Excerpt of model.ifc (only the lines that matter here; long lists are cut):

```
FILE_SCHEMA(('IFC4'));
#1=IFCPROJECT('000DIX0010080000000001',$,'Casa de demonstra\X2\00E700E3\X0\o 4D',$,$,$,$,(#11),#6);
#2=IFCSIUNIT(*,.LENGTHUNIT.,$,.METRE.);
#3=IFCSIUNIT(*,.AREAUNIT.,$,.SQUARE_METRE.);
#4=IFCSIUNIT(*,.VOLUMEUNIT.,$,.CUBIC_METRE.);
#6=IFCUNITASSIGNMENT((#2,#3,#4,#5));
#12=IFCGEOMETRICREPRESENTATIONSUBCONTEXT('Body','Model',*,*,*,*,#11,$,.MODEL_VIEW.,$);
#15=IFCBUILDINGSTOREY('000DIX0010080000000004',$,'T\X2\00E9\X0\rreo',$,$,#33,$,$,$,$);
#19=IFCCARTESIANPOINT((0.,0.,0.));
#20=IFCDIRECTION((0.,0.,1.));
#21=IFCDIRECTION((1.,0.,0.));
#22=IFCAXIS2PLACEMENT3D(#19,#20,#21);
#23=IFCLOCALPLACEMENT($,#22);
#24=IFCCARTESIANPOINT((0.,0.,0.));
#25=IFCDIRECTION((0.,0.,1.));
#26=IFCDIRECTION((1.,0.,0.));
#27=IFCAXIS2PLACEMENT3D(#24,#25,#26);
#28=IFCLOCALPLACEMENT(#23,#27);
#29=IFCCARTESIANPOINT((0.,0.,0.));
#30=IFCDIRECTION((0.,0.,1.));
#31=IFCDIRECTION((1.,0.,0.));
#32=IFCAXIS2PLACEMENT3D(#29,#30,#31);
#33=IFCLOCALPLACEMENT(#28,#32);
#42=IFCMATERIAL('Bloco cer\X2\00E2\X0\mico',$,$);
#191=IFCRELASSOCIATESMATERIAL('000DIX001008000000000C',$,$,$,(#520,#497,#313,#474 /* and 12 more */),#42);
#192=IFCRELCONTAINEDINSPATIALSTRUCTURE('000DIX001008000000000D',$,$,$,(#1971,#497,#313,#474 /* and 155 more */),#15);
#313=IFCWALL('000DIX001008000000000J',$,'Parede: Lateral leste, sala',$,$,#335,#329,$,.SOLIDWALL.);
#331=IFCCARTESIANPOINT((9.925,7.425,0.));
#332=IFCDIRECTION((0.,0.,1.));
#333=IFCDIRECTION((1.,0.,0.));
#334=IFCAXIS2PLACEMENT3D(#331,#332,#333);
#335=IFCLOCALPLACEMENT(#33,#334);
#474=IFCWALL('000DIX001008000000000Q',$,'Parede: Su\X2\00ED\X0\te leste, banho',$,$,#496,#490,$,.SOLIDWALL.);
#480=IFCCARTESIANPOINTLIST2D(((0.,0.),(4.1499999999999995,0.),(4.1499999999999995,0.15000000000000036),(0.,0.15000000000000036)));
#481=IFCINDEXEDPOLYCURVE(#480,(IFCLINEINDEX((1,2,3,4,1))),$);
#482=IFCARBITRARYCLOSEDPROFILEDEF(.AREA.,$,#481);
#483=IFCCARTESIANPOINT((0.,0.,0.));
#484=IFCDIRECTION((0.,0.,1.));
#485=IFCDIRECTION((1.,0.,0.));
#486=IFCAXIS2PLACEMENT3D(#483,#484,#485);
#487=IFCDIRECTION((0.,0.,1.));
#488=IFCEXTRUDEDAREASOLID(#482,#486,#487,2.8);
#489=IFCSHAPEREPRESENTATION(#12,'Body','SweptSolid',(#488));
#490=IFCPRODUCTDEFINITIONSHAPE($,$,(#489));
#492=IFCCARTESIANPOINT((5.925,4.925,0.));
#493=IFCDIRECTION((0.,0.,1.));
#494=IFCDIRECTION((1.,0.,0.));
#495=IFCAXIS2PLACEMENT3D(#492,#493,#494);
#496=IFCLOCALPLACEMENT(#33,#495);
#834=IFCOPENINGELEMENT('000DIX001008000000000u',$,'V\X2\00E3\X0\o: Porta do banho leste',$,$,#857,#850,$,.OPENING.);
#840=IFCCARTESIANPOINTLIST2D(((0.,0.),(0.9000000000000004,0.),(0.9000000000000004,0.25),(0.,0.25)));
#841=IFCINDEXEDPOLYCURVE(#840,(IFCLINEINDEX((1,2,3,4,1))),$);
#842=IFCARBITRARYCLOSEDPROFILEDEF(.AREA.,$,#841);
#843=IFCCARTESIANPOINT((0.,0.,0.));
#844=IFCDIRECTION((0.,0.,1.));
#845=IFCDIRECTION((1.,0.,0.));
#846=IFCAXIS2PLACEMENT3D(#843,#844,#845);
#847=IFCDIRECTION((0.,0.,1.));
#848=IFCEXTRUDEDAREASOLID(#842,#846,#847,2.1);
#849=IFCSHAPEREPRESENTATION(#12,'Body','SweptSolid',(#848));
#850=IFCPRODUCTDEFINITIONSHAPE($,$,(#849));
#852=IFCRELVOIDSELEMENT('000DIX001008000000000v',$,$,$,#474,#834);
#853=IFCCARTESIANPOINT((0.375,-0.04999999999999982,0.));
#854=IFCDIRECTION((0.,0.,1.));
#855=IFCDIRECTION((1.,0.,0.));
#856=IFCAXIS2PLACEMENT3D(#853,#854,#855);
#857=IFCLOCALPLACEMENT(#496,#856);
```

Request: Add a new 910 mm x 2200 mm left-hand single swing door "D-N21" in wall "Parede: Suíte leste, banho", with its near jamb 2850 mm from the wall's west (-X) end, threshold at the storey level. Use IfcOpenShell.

```python
import numpy as np
import ifcopenshell
import ifcopenshell.api.feature
import ifcopenshell.api.geometry
import ifcopenshell.api.root
import ifcopenshell.api.spatial
import ifcopenshell.geom
import ifcopenshell.util.element
import ifcopenshell.util.placement
import ifcopenshell.util.representation
import ifcopenshell.util.shape
import ifcopenshell.util.unit

model = ifcopenshell.open("model.ifc")
unit_scale = ifcopenshell.util.unit.calculate_unit_scale(model)
settings = ifcopenshell.geom.settings()


def volume(element):
    """Net volume in cubic metres, openings subtracted."""
    shape = ifcopenshell.geom.create_shape(settings, element)
    return ifcopenshell.util.shape.get_volume(shape.geometry)


wall = model.by_id(474)
storey = ifcopenshell.util.element.get_container(wall, ifc_class="IfcBuildingStorey")
context = ifcopenshell.util.representation.get_context(model, "Model", "Body", "MODEL_VIEW")
before = volume(wall)

width, height, from_end, sill = 0.91, 2.2, 2.85, 0.0  # metres

# The wall runs along its own X axis, and the end named is its -X end.
wall_shape = ifcopenshell.geom.create_shape(settings, wall)
x, y, z = ifcopenshell.util.shape.get_vertices(wall_shape.geometry).T
start = x.min() + from_end
face, thickness = float(y.min()), float(y.max() - y.min())
wall_matrix = ifcopenshell.util.placement.get_local_placement(wall.ObjectPlacement)
level = ifcopenshell.util.placement.get_local_placement(storey.ObjectPlacement)[2, 3]


def in_wall(x, y):
    """Placement at x, y metres in the wall's axes, at sill height."""
    matrix = wall_matrix.copy()
    matrix[:, 3] = wall_matrix @ np.array([x / unit_scale, y / unit_scale, 0.0, 1.0])
    matrix[2, 3] = level + sill / unit_scale
    return matrix


# Opening: a box that overshoots both wall faces by 50 mm.
opening = ifcopenshell.api.root.create_entity(model, ifc_class="IfcOpeningElement", predefined_type="OPENING")
box = ifcopenshell.api.geometry.add_wall_representation(
    model, context=context, length=width, height=height, thickness=thickness + 0.1
)
ifcopenshell.api.geometry.assign_representation(model, product=opening, representation=box)
ifcopenshell.api.geometry.edit_object_placement(model, product=opening, matrix=in_wall(start, face - 0.05), is_si=False)
ifcopenshell.api.feature.add_feature(model, feature=opening, element=wall)

door = ifcopenshell.api.root.create_entity(model, ifc_class="IfcDoor", name="D-N21", predefined_type="DOOR")
door.OverallWidth, door.OverallHeight = width / unit_scale, height / unit_scale
door.OperationType = "SINGLE_SWING_LEFT"
body = ifcopenshell.api.geometry.add_door_representation(
    model,
    context=context,
    overall_width=door.OverallWidth,
    overall_height=door.OverallHeight,
    operation_type="SINGLE_SWING_LEFT",
    lining_properties={"LiningDepth": thickness / unit_scale, "ThresholdDepth": thickness / unit_scale},
)
ifcopenshell.api.geometry.assign_representation(model, product=door, representation=body)
ifcopenshell.api.spatial.assign_container(model, products=[door], relating_structure=storey)
ifcopenshell.api.feature.add_filling(model, opening=opening, element=door)

# The lining spans the wall, so the door starts at the wall face.
ifcopenshell.api.geometry.edit_object_placement(model, product=door, matrix=in_wall(start, face), is_si=False)

after = volume(wall)

print(f"wall volume {before:.3f} -> {after:.3f} m3")

model.write("model_updated.ifc")
```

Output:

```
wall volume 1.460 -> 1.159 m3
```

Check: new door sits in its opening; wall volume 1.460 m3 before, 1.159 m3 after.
